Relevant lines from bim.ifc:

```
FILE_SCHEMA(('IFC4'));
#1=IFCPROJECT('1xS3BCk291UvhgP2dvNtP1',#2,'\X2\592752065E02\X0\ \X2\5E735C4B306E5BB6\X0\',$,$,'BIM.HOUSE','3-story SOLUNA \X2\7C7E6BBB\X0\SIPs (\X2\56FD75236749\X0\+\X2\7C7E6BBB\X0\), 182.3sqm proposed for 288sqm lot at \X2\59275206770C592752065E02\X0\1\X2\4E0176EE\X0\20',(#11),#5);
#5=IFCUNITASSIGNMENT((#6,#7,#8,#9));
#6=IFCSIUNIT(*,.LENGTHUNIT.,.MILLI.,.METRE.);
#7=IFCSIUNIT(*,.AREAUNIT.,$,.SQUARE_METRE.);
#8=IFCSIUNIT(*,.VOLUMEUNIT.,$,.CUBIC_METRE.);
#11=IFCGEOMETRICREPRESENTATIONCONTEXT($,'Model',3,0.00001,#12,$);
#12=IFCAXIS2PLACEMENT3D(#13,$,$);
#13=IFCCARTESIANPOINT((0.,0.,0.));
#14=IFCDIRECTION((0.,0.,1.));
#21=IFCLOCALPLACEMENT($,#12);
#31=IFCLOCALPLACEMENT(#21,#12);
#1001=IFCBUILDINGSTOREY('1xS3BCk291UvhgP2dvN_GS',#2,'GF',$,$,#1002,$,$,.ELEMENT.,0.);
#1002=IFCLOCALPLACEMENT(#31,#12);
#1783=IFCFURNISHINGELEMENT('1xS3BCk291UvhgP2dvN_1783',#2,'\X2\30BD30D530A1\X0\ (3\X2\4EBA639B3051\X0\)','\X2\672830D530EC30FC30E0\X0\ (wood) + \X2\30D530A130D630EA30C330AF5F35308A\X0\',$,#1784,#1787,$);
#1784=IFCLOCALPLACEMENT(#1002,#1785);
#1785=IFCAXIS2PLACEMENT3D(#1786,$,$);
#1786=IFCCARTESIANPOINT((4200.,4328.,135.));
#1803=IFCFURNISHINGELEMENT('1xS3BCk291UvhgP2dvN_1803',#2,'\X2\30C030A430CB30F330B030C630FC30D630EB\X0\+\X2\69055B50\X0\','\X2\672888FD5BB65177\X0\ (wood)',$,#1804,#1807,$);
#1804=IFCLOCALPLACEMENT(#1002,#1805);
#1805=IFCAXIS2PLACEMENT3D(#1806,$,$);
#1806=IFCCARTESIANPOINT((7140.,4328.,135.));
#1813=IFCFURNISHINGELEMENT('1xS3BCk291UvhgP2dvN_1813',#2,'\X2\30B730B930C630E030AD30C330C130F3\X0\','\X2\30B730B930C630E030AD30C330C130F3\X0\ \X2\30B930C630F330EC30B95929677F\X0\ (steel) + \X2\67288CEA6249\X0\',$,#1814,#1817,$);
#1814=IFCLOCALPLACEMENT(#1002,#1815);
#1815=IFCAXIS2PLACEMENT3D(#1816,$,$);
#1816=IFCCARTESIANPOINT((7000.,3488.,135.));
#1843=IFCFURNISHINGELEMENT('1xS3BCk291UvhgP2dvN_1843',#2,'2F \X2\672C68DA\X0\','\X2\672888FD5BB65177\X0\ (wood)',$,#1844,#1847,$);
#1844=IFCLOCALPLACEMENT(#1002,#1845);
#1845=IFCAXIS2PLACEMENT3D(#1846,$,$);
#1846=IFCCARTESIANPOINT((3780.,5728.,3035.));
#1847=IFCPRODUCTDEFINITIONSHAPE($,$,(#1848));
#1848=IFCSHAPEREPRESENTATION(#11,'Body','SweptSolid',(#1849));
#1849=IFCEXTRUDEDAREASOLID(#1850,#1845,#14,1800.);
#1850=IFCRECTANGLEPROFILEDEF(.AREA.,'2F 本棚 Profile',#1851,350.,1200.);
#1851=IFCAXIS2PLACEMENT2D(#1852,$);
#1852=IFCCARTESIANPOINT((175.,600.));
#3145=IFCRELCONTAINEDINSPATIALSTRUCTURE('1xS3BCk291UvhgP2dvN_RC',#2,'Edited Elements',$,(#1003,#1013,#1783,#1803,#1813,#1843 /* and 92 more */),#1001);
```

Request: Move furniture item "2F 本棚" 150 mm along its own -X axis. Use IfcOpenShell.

```python
import ifcopenshell
import ifcopenshell.api.geometry
import ifcopenshell.util.placement
import ifcopenshell.util.unit

model = ifcopenshell.open("bim.ifc")
unit_scale = ifcopenshell.util.unit.calculate_unit_scale(model)

item = model.by_guid("1xS3BCk291UvhgP2dvN_1843")
matrix = ifcopenshell.util.placement.get_local_placement(item.ObjectPlacement)
matrix[:3, 3] -= matrix[:3, 0] * 0.15 / unit_scale
ifcopenshell.api.geometry.edit_object_placement(model, product=item, matrix=matrix, is_si=False)

print(ifcopenshell.util.placement.get_local_placement(item.ObjectPlacement).round(3) + 0.0)

model.write("bim_updated.ifc")
```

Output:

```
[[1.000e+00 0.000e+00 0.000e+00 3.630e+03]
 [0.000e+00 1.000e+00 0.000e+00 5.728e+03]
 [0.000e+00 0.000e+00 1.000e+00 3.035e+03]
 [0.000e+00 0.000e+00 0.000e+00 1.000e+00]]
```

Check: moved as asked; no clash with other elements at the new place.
